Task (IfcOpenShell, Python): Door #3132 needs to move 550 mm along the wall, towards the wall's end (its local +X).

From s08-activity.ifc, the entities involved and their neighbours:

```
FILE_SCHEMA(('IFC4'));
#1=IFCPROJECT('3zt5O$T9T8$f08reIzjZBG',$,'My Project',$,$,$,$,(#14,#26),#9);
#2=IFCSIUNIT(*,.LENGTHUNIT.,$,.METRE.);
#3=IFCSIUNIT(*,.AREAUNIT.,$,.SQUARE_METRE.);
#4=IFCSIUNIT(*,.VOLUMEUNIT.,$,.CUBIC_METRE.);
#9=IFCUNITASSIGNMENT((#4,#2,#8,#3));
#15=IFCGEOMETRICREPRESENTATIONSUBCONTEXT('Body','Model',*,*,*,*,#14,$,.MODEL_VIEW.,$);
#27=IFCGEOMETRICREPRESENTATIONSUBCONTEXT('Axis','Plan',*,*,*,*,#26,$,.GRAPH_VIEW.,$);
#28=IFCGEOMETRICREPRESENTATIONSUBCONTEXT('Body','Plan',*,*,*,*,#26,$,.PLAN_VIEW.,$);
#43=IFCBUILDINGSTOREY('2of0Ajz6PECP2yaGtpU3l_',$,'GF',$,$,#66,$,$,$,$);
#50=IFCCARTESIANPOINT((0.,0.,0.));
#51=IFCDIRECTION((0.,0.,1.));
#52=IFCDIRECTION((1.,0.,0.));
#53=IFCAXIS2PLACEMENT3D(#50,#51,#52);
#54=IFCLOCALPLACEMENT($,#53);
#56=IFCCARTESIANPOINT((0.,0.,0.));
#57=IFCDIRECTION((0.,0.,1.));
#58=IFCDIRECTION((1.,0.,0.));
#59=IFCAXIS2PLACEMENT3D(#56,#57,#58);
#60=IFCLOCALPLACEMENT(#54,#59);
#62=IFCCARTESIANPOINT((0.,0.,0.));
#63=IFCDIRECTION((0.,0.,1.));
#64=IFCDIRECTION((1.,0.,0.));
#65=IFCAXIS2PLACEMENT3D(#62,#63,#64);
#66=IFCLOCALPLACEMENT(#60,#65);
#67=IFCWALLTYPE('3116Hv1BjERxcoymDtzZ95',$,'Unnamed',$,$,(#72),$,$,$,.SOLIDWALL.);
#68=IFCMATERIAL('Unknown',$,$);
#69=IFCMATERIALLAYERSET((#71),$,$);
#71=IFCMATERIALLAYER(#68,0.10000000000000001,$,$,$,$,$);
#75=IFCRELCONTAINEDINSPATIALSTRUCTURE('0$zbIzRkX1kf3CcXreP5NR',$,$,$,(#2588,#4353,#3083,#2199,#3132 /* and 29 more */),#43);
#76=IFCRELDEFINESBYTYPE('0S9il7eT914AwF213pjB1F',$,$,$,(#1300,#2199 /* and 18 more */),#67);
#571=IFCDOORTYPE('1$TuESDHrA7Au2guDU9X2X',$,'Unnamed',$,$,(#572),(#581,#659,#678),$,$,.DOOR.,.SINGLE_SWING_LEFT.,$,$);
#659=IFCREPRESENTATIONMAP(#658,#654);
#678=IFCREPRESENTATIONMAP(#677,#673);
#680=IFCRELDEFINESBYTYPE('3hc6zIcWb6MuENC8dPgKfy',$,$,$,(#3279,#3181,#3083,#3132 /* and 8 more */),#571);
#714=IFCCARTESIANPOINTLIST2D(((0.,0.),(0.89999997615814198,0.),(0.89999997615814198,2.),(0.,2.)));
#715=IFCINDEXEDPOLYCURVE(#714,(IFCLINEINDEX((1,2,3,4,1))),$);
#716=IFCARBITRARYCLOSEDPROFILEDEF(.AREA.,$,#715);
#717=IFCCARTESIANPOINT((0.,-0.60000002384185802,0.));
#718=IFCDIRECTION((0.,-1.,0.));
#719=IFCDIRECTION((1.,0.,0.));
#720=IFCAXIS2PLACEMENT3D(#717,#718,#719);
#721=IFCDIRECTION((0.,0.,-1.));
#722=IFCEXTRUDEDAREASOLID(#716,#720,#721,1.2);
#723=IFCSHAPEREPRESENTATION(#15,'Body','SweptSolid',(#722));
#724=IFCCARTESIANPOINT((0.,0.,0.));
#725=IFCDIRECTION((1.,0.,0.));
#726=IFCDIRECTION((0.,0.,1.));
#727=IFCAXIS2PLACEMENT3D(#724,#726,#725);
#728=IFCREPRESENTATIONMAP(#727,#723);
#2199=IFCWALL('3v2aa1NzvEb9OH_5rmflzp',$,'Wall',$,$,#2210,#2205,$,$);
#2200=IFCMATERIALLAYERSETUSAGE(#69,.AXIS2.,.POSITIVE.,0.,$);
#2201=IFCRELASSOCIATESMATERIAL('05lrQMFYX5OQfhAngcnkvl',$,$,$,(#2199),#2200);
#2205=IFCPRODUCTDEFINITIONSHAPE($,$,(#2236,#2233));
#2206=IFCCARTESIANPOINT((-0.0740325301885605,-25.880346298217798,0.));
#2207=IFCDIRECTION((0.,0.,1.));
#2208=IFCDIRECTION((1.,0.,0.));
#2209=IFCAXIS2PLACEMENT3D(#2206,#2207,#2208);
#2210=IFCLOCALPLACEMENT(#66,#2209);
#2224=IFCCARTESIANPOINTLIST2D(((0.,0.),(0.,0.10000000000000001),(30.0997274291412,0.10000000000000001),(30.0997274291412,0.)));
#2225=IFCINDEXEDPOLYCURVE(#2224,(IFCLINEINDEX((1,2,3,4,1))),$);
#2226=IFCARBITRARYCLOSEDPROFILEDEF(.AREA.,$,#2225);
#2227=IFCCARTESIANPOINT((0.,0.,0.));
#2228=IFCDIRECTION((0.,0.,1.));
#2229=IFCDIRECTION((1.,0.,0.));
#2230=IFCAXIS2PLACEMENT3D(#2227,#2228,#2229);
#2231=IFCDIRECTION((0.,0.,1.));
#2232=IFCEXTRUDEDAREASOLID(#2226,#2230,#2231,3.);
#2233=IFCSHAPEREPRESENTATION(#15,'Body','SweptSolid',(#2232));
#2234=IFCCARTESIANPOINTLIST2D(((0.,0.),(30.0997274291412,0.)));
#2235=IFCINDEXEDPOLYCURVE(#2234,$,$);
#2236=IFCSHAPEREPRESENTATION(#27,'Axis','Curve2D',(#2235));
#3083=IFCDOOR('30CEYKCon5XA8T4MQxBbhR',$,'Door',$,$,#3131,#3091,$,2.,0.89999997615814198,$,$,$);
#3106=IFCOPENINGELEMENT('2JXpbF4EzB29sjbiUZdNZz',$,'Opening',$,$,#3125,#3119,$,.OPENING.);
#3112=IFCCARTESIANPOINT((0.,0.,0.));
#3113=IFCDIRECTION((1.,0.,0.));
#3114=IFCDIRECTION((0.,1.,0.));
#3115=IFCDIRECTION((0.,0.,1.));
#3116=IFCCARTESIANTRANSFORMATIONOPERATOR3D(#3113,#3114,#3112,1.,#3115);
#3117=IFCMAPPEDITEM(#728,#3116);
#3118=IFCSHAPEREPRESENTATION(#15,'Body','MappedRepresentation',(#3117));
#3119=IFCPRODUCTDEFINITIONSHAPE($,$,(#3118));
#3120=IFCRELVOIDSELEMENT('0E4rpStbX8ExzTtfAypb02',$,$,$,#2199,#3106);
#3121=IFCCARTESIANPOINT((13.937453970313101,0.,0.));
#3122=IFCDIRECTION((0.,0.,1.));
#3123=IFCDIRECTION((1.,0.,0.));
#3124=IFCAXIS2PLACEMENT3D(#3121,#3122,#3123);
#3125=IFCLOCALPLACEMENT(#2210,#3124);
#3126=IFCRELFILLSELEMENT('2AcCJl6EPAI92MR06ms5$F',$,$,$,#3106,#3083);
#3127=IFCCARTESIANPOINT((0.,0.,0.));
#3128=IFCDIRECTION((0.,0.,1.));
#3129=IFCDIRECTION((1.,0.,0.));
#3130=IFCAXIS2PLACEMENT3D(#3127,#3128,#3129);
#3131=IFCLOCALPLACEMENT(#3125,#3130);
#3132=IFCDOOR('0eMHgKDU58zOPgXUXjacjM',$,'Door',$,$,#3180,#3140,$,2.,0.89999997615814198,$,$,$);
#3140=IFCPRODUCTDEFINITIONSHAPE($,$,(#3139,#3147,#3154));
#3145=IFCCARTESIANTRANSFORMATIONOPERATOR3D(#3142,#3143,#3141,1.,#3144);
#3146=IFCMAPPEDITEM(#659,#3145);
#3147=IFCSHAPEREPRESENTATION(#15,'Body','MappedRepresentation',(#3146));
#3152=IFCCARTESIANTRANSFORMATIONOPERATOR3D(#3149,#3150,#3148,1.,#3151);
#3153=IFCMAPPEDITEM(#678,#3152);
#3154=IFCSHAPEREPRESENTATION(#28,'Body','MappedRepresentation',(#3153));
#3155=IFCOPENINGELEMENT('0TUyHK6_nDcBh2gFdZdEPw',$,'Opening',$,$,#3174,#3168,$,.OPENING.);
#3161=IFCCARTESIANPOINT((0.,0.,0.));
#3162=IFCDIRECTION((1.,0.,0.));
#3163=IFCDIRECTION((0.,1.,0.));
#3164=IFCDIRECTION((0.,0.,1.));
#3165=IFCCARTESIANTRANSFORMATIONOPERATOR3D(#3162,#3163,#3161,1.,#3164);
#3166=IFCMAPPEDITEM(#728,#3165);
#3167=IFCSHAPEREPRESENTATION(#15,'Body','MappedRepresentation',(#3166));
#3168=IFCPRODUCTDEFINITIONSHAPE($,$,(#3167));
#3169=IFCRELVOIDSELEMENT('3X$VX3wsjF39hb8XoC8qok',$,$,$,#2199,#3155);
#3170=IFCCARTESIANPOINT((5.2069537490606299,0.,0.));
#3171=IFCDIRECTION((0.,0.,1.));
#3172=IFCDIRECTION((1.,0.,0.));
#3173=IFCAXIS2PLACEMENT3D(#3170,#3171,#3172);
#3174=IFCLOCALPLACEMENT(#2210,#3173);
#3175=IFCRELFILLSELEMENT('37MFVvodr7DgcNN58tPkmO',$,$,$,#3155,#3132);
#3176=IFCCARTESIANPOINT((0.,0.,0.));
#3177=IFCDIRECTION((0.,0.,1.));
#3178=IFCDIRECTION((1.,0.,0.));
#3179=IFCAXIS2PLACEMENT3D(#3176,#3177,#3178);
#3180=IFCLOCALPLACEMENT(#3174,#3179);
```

```python
import ifcopenshell
import ifcopenshell.api.geometry
import ifcopenshell.util.placement

model = ifcopenshell.open("s08-activity.ifc")

door = model.by_guid("0eMHgKDU58zOPgXUXjacjM")
opening = door.FillsVoids[0].RelatingOpeningElement
wall = opening.VoidsElements[0].RelatingBuildingElement

wall_matrix = ifcopenshell.util.placement.get_local_placement(wall.ObjectPlacement)
shift = wall_matrix[:3, 0] * 0.55
before = ifcopenshell.util.placement.get_local_placement(door.ObjectPlacement)[:3, 3].copy()

# The door is placed relative to its opening, so it follows when the opening moves.
matrix = ifcopenshell.util.placement.get_local_placement(opening.ObjectPlacement)
matrix[:3, 3] += shift
ifcopenshell.api.geometry.edit_object_placement(
    model, product=opening, matrix=matrix, is_si=False, should_transform_children=True
)

after = ifcopenshell.util.placement.get_local_placement(door.ObjectPlacement)[:3, 3]
print("door moved by", (after - before).round(3) + 0.0)

model.write("s08-activity_updated.ifc")
```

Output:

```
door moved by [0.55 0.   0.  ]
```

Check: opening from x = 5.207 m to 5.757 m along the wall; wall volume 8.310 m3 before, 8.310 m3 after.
